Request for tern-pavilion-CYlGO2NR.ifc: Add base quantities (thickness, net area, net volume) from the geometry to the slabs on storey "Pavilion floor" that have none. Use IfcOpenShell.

First a look at what the model holds.

```python
import ifcopenshell
import ifcopenshell.util.element
import ifcopenshell.util.unit

model = ifcopenshell.open("tern-pavilion-CYlGO2NR.ifc")
print(model.schema)
for unit_type in ("LENGTHUNIT", "AREAUNIT", "VOLUMEUNIT"):
    print(unit_type, ifcopenshell.util.unit.calculate_unit_scale(model, unit_type))
storey = next(s for s in model.by_type("IfcBuildingStorey") if s.Name == "Pavilion floor")
slabs = [e for e in ifcopenshell.util.element.get_decomposition(storey) if e.is_a("IfcSlab")]
for e in sorted(slabs, key=lambda e: e.id()):
    print(e.id(), e.is_a(), e.Name, list(ifcopenshell.util.element.get_psets(e, qtos_only=True)), sep=" | ")
```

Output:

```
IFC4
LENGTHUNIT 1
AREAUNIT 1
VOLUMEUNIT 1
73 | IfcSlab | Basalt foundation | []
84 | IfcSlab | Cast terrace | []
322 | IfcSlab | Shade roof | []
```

```python
import ifcopenshell
import ifcopenshell.api.pset
import ifcopenshell.geom
import ifcopenshell.util.element
import ifcopenshell.util.shape
import ifcopenshell.util.unit

model = ifcopenshell.open("tern-pavilion-CYlGO2NR.ifc")
unit_scale = ifcopenshell.util.unit.calculate_unit_scale(model)
area_scale = ifcopenshell.util.unit.calculate_unit_scale(model, "AREAUNIT")
volume_scale = ifcopenshell.util.unit.calculate_unit_scale(model, "VOLUMEUNIT")
settings = ifcopenshell.geom.settings()

storey = next(s for s in model.by_type("IfcBuildingStorey") if s.Name == "Pavilion floor")
slabs = [e for e in ifcopenshell.util.element.get_decomposition(storey) if e.is_a("IfcSlab")]

for e in sorted(slabs, key=lambda e: e.id()):
    if ifcopenshell.util.element.get_psets(e, qtos_only=True, should_inherit=False):
        continue
    # Geometry comes back in metres, in the element's own axes.
    shape = ifcopenshell.geom.create_shape(settings, e)
    values = {
        "Width": ifcopenshell.util.shape.get_z(shape.geometry) / unit_scale,
        "NetArea": ifcopenshell.util.shape.get_footprint_area(shape.geometry) / area_scale,
        "NetVolume": ifcopenshell.util.shape.get_volume(shape.geometry) / volume_scale,
    }
    qto = ifcopenshell.api.pset.add_qto(model, product=e, name="Qto_SlabBaseQuantities")
    ifcopenshell.api.pset.edit_qto(model, qto=qto, properties=values)
    print(e.id(), {k: round(v, 3) for k, v in values.items()})

model.write("tern-pavilion-CYlGO2NR_rev.ifc")
```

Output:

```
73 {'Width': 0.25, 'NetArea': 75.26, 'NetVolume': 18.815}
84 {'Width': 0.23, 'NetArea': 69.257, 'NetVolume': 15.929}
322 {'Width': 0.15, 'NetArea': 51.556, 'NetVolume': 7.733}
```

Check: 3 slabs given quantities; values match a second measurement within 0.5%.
